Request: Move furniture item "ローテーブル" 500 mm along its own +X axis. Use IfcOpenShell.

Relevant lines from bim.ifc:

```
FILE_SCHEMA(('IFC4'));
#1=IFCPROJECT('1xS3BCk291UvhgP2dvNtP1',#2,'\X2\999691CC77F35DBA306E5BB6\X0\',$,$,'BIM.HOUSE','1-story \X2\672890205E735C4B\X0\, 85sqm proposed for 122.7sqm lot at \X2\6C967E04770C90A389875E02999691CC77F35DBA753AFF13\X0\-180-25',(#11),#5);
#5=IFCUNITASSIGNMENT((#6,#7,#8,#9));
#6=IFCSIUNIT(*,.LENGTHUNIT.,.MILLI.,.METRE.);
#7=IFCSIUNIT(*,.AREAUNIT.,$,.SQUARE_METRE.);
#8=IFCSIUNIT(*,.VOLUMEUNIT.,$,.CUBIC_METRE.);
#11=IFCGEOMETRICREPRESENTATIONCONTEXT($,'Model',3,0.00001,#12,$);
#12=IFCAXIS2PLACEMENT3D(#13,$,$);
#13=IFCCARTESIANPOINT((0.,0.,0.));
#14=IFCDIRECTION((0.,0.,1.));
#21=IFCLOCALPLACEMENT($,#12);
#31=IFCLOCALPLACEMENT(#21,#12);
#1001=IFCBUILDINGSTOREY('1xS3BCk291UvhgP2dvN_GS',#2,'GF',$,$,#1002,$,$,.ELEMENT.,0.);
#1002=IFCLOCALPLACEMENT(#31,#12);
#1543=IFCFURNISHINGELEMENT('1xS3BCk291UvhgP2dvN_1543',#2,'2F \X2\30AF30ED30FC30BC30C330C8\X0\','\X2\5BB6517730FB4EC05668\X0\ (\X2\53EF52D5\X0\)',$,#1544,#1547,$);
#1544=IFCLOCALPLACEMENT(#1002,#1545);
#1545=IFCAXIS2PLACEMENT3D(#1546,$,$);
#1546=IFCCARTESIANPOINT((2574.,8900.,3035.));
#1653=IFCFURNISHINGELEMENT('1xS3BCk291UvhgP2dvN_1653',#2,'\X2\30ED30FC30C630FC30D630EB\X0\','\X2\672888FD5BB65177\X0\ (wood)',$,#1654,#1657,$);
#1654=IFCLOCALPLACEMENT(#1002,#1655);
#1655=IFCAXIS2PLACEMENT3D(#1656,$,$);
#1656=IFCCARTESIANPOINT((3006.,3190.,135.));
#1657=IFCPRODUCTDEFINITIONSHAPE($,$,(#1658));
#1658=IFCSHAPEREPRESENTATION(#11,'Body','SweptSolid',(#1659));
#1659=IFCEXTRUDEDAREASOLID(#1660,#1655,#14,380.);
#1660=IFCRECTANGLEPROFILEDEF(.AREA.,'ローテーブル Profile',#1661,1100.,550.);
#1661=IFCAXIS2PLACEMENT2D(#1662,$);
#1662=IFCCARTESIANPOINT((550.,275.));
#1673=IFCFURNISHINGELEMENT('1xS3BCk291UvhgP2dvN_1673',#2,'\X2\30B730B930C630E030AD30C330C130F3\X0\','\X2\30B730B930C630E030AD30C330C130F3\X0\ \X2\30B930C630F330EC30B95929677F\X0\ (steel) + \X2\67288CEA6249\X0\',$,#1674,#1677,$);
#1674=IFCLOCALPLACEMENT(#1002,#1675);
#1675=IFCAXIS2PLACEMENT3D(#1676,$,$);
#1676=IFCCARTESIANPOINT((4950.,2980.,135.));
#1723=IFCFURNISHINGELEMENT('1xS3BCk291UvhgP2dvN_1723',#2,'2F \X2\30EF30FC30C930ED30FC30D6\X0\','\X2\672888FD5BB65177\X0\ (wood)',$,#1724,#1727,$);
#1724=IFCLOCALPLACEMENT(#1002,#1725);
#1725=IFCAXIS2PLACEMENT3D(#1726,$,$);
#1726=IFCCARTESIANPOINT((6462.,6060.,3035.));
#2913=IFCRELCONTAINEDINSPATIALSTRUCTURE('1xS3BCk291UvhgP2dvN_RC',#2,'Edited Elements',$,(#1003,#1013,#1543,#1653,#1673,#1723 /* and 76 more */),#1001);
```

```python
import ifcopenshell
import ifcopenshell.api.geometry
import ifcopenshell.util.placement
import ifcopenshell.util.unit

model = ifcopenshell.open("bim.ifc")
unit_scale = ifcopenshell.util.unit.calculate_unit_scale(model)

item = model.by_id(1653)
matrix = ifcopenshell.util.placement.get_local_placement(item.ObjectPlacement)
matrix[:3, 3] += matrix[:3, 0] * 0.5 / unit_scale
ifcopenshell.api.geometry.edit_object_placement(model, product=item, matrix=matrix, is_si=False)

print(ifcopenshell.util.placement.get_local_placement(item.ObjectPlacement).round(3) + 0.0)

model.write("bim_edited.ifc")
```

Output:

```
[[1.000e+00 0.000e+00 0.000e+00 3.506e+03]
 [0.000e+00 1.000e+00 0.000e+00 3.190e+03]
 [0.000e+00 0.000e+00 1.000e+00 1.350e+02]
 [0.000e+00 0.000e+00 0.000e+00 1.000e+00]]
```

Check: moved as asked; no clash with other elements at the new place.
